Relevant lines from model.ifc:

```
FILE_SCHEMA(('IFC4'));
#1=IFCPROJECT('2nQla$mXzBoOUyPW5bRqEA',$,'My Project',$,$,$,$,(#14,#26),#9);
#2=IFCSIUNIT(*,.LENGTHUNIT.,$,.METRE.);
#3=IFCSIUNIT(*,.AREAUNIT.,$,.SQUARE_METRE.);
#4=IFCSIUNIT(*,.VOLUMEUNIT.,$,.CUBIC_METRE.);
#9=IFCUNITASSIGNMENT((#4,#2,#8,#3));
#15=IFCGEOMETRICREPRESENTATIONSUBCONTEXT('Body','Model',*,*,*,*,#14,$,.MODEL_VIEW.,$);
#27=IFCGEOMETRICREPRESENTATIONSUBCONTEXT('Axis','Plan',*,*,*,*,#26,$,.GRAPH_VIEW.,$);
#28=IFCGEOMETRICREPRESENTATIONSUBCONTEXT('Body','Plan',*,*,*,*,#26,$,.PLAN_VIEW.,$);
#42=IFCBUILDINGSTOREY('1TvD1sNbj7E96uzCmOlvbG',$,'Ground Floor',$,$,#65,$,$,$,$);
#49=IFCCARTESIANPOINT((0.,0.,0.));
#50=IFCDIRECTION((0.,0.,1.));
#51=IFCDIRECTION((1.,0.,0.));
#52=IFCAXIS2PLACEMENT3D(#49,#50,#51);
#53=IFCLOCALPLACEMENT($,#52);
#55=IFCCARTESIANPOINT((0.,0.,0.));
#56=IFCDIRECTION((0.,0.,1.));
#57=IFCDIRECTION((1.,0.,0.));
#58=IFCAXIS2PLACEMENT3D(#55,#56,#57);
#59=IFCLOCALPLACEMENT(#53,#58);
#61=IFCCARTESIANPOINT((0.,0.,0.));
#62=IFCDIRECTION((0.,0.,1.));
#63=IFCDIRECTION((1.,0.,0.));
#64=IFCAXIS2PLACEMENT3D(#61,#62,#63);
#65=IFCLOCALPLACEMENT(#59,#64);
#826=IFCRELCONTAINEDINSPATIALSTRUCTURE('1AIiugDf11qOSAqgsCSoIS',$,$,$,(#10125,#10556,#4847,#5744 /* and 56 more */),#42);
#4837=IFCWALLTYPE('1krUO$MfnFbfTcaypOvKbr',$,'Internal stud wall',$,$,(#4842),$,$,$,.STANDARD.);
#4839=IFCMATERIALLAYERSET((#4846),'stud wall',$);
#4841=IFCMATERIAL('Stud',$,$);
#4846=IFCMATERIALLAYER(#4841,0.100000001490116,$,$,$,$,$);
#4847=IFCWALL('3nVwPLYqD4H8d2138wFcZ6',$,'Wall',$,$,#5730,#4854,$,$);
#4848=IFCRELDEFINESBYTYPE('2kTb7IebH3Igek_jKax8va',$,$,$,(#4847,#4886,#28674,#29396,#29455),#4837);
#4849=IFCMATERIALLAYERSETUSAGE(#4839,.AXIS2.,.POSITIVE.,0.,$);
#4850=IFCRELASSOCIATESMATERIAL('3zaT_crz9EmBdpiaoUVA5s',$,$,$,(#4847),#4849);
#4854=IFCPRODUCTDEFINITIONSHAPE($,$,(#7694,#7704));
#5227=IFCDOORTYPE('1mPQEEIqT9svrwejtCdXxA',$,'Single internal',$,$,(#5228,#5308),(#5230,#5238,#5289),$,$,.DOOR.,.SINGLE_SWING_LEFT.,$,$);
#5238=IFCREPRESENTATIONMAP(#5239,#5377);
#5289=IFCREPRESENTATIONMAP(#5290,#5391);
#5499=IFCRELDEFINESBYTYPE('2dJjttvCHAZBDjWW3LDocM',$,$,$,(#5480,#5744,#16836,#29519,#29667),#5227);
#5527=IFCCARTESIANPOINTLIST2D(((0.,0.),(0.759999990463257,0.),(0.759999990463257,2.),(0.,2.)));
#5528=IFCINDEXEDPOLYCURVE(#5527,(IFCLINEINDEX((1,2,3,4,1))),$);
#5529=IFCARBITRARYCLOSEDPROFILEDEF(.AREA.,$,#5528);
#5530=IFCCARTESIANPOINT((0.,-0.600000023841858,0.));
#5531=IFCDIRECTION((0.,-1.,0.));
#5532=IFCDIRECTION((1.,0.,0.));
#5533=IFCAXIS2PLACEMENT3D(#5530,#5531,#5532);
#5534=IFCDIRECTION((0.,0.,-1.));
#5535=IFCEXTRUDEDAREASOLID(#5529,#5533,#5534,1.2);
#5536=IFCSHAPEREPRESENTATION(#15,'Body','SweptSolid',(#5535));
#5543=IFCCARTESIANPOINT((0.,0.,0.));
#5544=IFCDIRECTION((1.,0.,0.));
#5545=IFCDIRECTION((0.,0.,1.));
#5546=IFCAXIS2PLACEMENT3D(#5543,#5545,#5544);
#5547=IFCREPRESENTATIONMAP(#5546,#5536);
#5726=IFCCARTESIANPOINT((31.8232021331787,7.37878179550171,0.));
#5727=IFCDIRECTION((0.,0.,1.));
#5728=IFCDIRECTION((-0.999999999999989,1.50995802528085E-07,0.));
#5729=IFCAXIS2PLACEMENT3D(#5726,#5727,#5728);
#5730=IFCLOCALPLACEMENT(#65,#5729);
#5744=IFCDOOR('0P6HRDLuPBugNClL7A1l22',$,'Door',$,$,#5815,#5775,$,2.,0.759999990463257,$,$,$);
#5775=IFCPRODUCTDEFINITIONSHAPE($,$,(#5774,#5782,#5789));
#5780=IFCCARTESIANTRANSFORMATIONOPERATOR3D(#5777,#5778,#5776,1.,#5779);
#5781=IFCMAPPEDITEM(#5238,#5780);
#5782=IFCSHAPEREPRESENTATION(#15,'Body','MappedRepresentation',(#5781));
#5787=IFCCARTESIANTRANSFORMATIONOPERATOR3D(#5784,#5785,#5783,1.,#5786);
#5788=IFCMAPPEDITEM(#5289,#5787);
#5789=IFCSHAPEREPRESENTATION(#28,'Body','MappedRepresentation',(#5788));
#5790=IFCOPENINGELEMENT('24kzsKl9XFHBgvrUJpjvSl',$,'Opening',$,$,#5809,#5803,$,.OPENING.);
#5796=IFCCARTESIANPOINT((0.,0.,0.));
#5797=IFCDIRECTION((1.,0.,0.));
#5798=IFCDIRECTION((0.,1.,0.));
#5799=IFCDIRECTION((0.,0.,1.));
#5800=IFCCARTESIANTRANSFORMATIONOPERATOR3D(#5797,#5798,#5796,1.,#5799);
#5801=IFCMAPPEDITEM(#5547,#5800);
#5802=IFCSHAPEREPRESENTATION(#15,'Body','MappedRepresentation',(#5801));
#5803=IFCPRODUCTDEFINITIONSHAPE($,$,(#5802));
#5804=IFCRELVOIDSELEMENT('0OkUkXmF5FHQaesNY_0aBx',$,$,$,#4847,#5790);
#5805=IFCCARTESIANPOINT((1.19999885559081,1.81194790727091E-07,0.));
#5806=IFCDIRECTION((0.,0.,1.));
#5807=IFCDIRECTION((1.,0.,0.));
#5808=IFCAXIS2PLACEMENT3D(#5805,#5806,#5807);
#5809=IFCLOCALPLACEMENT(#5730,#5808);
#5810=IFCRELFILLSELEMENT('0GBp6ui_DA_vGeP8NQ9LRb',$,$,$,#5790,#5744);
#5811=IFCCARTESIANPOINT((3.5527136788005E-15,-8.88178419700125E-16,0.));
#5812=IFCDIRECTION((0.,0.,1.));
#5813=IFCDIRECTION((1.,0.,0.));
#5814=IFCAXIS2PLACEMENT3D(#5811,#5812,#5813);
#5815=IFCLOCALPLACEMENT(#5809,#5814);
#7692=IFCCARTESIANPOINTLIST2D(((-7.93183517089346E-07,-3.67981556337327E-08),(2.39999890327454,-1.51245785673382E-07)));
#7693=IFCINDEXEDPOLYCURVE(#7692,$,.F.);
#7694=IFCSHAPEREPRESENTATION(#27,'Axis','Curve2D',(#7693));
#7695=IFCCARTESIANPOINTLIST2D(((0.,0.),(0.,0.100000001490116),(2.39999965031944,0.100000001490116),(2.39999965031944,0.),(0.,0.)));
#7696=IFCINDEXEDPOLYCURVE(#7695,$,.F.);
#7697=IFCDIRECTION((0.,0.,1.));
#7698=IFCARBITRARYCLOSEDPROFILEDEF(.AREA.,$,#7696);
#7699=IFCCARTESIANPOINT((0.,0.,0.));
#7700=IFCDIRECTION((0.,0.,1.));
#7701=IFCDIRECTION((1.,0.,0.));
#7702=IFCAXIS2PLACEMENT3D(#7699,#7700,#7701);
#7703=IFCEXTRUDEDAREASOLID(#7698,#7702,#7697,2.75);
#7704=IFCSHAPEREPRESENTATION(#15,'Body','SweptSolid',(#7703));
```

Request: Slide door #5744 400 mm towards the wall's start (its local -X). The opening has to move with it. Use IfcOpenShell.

```python
import ifcopenshell
import ifcopenshell.api.geometry
import ifcopenshell.util.placement

model = ifcopenshell.open("model.ifc")

door = model.by_guid("0P6HRDLuPBugNClL7A1l22")
opening = door.FillsVoids[0].RelatingOpeningElement
wall = opening.VoidsElements[0].RelatingBuildingElement

wall_matrix = ifcopenshell.util.placement.get_local_placement(wall.ObjectPlacement)
shift = wall_matrix[:3, 0] * -0.4
before = ifcopenshell.util.placement.get_local_placement(door.ObjectPlacement)[:3, 3].copy()

# The door is placed relative to its opening, so it follows when the opening moves.
matrix = ifcopenshell.util.placement.get_local_placement(opening.ObjectPlacement)
matrix[:3, 3] += shift
ifcopenshell.api.geometry.edit_object_placement(
    model, product=opening, matrix=matrix, is_si=False, should_transform_children=True
)

after = ifcopenshell.util.placement.get_local_placement(door.ObjectPlacement)[:3, 3]
print("door moved by", (after - before).round(3) + 0.0)

model.write("model_v2.ifc")
```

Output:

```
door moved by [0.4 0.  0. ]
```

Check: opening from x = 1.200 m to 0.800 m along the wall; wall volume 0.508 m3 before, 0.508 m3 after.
